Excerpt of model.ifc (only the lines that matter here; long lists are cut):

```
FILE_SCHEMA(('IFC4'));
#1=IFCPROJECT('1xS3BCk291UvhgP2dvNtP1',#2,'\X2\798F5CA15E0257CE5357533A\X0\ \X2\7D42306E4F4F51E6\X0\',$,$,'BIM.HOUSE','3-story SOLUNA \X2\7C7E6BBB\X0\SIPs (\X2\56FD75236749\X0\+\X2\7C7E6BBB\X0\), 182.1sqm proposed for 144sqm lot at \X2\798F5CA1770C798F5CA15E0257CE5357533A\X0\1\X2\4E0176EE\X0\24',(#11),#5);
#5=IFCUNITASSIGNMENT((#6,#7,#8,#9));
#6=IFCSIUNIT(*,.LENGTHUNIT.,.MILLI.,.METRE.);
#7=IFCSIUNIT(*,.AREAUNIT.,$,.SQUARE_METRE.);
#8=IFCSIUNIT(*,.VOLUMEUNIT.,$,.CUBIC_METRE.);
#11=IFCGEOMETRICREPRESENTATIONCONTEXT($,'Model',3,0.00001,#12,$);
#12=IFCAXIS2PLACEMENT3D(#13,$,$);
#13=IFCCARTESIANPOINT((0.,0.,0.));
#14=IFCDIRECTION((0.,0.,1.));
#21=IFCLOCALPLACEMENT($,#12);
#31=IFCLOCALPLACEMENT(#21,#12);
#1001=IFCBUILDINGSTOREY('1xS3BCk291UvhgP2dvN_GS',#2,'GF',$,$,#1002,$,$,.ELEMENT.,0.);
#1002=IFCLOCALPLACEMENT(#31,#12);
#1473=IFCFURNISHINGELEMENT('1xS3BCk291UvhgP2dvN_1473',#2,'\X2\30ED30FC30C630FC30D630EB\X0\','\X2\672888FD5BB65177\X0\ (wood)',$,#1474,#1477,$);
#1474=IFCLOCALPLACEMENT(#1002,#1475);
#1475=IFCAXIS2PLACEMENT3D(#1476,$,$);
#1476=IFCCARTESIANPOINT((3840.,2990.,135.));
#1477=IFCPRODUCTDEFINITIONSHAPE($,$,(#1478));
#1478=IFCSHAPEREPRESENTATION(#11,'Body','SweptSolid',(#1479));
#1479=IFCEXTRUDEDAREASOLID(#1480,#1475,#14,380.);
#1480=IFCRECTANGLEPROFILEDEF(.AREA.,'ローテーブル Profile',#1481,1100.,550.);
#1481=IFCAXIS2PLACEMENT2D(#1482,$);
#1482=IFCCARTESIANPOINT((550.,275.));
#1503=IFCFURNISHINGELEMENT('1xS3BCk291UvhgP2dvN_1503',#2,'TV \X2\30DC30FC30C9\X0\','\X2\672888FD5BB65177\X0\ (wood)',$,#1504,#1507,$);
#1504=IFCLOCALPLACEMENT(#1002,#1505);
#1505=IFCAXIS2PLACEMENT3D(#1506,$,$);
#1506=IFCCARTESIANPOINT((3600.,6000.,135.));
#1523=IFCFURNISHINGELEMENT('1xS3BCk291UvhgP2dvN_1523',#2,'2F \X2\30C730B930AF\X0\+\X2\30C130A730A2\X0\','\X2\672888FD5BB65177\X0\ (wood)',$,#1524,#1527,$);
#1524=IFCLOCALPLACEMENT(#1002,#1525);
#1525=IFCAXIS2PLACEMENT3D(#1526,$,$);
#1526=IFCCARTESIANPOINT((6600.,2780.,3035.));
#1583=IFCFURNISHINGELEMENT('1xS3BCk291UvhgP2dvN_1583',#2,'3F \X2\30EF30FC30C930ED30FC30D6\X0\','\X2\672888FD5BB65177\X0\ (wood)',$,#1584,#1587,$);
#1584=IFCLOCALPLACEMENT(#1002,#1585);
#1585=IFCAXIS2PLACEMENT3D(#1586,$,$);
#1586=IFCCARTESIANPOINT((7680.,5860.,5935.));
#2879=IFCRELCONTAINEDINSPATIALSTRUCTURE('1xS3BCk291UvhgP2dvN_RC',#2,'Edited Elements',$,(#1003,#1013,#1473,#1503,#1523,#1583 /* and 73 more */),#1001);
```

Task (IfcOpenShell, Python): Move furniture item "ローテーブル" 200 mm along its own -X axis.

```python
import ifcopenshell
import ifcopenshell.api.geometry
import ifcopenshell.util.placement
import ifcopenshell.util.unit

model = ifcopenshell.open("model.ifc")
unit_scale = ifcopenshell.util.unit.calculate_unit_scale(model)

item = model.by_guid("1xS3BCk291UvhgP2dvN_1473")
matrix = ifcopenshell.util.placement.get_local_placement(item.ObjectPlacement)
matrix[:3, 3] -= matrix[:3, 0] * 0.2 / unit_scale
ifcopenshell.api.geometry.edit_object_placement(model, product=item, matrix=matrix, is_si=False)

print(ifcopenshell.util.placement.get_local_placement(item.ObjectPlacement).round(3) + 0.0)

model.write("model_updated.ifc")
```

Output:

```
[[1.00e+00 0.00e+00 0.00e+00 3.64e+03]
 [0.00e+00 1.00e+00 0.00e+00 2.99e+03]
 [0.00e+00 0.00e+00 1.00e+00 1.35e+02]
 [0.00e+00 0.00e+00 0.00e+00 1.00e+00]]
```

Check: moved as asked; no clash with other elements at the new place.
